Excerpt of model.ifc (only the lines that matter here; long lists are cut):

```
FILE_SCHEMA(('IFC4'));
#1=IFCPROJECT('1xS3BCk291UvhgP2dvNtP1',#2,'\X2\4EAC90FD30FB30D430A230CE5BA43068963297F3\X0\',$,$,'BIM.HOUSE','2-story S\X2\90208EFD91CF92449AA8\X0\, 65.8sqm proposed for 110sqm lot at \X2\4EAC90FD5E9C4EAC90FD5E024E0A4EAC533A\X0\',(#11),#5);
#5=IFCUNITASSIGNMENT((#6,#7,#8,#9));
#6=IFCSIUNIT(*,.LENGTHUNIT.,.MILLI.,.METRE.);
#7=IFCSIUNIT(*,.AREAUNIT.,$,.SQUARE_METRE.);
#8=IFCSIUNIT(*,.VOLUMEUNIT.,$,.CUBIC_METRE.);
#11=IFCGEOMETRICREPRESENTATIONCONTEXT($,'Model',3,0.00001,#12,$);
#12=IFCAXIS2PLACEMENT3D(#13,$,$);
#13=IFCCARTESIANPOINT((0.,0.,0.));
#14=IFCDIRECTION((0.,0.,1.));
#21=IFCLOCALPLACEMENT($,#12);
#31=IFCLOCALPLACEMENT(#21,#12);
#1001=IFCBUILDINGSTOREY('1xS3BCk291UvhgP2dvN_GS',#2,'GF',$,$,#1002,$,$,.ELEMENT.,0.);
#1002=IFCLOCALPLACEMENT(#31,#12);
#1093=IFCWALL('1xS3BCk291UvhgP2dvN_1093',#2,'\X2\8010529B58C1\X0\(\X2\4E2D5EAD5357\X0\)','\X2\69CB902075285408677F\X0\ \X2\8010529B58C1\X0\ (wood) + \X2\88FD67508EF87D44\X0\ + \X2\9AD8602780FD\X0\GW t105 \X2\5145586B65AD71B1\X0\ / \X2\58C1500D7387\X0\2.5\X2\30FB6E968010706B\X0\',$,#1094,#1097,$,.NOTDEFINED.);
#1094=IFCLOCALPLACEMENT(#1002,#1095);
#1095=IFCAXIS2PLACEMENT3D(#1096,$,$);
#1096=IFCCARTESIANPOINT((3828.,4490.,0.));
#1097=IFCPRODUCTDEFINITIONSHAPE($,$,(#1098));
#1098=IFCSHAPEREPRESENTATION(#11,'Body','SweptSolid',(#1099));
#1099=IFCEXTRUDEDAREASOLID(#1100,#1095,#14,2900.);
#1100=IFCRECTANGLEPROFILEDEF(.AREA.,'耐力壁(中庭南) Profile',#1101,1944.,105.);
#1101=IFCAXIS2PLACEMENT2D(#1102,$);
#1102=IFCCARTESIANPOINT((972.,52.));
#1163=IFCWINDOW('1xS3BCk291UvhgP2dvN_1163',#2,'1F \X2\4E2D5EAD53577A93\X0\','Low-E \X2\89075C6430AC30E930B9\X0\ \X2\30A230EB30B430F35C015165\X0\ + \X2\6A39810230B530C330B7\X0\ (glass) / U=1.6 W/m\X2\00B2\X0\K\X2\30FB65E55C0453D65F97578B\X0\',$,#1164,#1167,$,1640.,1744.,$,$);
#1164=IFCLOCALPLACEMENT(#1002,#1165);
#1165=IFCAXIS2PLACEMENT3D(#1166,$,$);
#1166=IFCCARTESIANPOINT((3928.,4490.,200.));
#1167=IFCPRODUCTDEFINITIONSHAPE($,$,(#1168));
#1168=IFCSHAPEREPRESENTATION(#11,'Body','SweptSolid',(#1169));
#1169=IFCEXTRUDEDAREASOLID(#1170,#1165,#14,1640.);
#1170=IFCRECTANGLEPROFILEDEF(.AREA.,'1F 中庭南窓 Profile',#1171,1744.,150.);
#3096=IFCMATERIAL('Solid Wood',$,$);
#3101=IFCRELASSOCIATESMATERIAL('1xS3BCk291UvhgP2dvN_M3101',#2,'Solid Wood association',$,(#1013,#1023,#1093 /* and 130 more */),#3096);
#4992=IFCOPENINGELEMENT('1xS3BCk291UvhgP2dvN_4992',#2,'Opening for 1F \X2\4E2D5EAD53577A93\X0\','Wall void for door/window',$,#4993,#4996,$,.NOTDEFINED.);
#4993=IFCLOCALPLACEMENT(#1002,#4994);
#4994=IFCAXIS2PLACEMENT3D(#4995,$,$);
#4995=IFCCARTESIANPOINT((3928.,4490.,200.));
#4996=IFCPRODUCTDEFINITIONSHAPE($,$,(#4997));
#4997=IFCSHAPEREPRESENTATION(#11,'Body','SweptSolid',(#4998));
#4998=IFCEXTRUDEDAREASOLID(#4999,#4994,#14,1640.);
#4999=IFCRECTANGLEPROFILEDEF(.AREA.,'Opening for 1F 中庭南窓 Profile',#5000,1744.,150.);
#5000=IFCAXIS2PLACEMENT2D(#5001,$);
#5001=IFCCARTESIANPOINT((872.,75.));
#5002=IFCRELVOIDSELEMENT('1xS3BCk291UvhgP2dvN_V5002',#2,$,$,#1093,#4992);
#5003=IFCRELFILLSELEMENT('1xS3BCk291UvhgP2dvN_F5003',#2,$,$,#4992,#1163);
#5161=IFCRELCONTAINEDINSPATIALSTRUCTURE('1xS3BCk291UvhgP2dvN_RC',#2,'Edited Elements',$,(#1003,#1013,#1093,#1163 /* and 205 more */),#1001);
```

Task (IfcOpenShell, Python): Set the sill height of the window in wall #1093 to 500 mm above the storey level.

```python
import numpy as np
import ifcopenshell
import ifcopenshell.api.geometry
import ifcopenshell.geom
import ifcopenshell.util.element
import ifcopenshell.util.placement
import ifcopenshell.util.shape
import ifcopenshell.util.unit

model = ifcopenshell.open("model.ifc")
unit_scale = ifcopenshell.util.unit.calculate_unit_scale(model)

window = model.by_guid("1xS3BCk291UvhgP2dvN_1163")
opening = window.FillsVoids[0].RelatingOpeningElement
storey = ifcopenshell.util.element.get_container(window, ifc_class="IfcBuildingStorey")
level = ifcopenshell.util.placement.get_local_placement(storey.ObjectPlacement)[2, 3]

# The opening's origin need not be at the sill, so measure its lowest point.
shape = ifcopenshell.geom.create_shape(ifcopenshell.geom.settings(), opening)
bottom = ifcopenshell.util.shape.get_shape_bottom_elevation(shape, shape.geometry) / unit_scale
dz = level + 0.5 / unit_scale - bottom

shift = np.array([0.0, 0.0, dz])
# The window is not placed relative to its opening, so move both.
for product in (opening, window):
    matrix = ifcopenshell.util.placement.get_local_placement(product.ObjectPlacement)
    matrix[:3, 3] += shift
    ifcopenshell.api.geometry.edit_object_placement(model, product=product, matrix=matrix, is_si=False)

print(f"moved by {dz * unit_scale:+.3f} m")

model.write("model_updated.ifc")
```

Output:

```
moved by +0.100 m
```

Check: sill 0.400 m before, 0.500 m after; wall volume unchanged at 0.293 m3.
